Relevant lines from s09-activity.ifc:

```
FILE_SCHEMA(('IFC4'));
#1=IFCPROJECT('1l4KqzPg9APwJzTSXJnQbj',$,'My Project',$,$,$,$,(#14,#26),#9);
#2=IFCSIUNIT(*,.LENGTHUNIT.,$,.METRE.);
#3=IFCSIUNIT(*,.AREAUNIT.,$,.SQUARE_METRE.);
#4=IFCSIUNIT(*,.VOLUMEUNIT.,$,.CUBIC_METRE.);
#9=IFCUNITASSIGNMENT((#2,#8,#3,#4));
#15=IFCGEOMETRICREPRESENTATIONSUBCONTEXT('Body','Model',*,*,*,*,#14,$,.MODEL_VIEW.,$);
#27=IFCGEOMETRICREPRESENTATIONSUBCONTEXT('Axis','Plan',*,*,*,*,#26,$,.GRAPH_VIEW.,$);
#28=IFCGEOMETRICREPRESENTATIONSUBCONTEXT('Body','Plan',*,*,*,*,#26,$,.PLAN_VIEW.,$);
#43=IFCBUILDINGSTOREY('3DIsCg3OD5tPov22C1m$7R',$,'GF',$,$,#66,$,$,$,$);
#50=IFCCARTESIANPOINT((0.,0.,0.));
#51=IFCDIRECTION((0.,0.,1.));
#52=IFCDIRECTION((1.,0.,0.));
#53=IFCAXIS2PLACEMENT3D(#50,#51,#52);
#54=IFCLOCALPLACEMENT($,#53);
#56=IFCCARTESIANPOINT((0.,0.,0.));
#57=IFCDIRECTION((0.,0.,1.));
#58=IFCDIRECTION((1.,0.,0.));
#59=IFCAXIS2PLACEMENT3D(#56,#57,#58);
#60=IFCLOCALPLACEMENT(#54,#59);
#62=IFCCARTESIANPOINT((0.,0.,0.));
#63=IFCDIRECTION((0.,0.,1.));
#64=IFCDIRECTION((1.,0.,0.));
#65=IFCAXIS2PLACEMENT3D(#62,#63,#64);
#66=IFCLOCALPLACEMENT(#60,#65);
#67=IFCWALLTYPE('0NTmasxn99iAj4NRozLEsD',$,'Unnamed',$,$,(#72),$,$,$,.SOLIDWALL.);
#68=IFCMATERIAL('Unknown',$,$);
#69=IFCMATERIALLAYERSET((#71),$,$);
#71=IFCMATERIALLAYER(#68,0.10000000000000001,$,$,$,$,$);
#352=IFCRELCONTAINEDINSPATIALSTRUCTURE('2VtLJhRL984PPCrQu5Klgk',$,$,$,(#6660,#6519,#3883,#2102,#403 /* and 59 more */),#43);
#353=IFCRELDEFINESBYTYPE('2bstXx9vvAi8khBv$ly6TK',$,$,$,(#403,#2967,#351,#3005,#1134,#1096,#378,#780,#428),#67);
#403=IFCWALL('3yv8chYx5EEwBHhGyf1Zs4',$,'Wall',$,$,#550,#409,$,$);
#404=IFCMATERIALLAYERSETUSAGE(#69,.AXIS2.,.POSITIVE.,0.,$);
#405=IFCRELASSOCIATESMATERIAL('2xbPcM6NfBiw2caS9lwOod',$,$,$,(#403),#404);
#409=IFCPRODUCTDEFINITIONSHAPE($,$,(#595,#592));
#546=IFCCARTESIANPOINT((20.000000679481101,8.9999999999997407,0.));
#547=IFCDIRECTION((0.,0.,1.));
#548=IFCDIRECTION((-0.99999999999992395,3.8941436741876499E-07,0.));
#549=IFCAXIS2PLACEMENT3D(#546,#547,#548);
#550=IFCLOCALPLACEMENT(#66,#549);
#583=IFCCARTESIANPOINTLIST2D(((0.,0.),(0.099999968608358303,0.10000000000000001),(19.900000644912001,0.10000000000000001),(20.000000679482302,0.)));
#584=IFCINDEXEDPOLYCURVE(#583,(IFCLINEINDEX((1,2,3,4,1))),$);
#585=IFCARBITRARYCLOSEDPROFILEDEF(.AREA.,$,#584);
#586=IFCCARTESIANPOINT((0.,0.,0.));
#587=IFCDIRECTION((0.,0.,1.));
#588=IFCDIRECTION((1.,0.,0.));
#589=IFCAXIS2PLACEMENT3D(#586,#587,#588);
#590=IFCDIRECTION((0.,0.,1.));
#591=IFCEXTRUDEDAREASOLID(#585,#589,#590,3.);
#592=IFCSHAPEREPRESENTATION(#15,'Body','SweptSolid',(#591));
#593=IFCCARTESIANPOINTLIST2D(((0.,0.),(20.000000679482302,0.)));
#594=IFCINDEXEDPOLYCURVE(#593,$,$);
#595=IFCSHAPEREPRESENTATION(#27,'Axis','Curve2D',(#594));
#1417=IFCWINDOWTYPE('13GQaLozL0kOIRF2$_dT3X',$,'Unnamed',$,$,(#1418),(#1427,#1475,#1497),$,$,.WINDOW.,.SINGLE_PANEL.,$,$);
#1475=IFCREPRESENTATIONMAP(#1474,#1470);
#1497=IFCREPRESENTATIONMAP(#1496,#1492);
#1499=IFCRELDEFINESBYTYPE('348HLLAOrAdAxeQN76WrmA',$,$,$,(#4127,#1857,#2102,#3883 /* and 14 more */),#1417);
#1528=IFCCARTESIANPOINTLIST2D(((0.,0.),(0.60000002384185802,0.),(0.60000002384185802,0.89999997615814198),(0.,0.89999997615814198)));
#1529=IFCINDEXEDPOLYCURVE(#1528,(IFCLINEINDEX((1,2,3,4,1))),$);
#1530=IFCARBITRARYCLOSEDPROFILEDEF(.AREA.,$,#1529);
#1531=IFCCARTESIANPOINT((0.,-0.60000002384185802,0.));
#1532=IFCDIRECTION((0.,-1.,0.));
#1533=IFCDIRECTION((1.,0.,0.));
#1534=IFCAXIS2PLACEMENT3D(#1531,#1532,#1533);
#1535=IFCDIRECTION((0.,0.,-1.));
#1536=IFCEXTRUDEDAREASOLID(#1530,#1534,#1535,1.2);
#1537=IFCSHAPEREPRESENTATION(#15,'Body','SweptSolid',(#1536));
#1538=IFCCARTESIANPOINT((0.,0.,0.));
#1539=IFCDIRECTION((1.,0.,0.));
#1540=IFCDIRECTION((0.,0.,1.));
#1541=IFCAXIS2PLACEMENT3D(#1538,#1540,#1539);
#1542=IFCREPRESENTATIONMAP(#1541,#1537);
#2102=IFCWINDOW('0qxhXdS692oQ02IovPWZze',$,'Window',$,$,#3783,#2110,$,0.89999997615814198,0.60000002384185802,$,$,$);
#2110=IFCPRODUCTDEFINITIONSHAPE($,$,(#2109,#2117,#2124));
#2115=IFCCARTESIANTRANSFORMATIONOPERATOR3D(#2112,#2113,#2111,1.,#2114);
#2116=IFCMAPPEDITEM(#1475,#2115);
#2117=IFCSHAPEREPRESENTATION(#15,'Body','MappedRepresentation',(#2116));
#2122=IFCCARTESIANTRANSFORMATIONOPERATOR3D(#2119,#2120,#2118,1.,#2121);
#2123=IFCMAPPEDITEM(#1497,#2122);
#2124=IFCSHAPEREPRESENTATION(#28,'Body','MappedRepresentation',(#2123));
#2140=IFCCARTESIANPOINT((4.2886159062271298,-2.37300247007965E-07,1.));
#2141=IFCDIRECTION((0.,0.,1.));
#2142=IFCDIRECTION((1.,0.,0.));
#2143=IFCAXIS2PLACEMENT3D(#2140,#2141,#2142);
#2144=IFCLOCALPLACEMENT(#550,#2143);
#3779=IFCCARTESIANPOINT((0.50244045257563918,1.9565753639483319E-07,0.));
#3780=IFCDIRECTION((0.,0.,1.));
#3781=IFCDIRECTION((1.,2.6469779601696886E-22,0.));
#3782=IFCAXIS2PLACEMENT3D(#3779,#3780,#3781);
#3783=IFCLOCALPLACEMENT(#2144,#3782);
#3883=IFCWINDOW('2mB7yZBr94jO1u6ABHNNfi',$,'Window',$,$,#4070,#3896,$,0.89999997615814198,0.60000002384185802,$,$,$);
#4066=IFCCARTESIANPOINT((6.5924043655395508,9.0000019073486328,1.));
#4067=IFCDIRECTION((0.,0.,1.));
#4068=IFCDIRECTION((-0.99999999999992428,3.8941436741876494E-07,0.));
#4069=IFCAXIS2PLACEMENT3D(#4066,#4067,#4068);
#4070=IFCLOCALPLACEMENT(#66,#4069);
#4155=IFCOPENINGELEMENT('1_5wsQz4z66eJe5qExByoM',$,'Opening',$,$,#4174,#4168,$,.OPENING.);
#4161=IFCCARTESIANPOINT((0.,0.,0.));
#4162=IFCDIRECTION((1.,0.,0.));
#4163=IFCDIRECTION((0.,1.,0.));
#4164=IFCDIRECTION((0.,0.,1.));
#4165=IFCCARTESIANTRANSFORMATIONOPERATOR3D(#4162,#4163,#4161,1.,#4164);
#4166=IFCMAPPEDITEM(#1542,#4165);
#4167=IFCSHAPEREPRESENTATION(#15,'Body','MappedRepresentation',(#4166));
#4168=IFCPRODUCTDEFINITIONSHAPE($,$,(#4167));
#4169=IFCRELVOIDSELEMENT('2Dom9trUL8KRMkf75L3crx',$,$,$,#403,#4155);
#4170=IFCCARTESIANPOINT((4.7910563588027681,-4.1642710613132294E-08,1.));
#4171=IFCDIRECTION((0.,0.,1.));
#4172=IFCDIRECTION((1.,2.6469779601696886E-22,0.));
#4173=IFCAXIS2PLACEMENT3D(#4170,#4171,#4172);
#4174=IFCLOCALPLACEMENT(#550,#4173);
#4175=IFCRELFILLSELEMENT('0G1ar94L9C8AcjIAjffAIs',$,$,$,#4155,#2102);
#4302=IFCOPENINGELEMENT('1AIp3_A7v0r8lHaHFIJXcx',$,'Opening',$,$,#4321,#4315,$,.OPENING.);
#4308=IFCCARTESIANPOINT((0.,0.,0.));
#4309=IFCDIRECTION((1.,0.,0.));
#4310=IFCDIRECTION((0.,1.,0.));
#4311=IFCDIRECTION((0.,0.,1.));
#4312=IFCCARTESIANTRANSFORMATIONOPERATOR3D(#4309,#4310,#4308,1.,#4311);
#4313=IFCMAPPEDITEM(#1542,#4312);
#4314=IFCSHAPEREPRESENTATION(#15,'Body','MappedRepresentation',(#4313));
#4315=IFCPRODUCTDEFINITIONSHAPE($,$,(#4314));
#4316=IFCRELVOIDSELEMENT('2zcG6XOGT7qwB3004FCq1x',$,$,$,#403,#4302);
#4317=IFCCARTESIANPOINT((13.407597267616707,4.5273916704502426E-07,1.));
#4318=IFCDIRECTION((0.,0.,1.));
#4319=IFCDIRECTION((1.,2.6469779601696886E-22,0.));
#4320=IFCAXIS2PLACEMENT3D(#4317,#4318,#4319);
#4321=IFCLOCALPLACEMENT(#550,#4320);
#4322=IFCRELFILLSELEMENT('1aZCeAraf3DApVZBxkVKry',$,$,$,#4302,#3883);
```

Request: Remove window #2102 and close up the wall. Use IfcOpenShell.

```python
import ifcopenshell
import ifcopenshell.api.feature
import ifcopenshell.api.root
import ifcopenshell.geom
import ifcopenshell.util.shape

model = ifcopenshell.open("s09-activity.ifc")
settings = ifcopenshell.geom.settings()


def volume(element):
    """Net volume in cubic metres, openings subtracted."""
    shape = ifcopenshell.geom.create_shape(settings, element)
    return ifcopenshell.util.shape.get_volume(shape.geometry)


window = model.by_guid("0qxhXdS692oQ02IovPWZze")
opening = window.FillsVoids[0].RelatingOpeningElement
wall = opening.VoidsElements[0].RelatingBuildingElement
before = volume(wall)

ifcopenshell.api.root.remove_product(model, product=window)
ifcopenshell.api.feature.remove_feature(model, feature=opening)

after = volume(wall)

print(f"wall volume {before:.3f} -> {after:.3f} m3")

model.write("s09-activity_rev.ifc")
```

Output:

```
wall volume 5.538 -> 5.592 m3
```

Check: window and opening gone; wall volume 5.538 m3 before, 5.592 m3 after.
